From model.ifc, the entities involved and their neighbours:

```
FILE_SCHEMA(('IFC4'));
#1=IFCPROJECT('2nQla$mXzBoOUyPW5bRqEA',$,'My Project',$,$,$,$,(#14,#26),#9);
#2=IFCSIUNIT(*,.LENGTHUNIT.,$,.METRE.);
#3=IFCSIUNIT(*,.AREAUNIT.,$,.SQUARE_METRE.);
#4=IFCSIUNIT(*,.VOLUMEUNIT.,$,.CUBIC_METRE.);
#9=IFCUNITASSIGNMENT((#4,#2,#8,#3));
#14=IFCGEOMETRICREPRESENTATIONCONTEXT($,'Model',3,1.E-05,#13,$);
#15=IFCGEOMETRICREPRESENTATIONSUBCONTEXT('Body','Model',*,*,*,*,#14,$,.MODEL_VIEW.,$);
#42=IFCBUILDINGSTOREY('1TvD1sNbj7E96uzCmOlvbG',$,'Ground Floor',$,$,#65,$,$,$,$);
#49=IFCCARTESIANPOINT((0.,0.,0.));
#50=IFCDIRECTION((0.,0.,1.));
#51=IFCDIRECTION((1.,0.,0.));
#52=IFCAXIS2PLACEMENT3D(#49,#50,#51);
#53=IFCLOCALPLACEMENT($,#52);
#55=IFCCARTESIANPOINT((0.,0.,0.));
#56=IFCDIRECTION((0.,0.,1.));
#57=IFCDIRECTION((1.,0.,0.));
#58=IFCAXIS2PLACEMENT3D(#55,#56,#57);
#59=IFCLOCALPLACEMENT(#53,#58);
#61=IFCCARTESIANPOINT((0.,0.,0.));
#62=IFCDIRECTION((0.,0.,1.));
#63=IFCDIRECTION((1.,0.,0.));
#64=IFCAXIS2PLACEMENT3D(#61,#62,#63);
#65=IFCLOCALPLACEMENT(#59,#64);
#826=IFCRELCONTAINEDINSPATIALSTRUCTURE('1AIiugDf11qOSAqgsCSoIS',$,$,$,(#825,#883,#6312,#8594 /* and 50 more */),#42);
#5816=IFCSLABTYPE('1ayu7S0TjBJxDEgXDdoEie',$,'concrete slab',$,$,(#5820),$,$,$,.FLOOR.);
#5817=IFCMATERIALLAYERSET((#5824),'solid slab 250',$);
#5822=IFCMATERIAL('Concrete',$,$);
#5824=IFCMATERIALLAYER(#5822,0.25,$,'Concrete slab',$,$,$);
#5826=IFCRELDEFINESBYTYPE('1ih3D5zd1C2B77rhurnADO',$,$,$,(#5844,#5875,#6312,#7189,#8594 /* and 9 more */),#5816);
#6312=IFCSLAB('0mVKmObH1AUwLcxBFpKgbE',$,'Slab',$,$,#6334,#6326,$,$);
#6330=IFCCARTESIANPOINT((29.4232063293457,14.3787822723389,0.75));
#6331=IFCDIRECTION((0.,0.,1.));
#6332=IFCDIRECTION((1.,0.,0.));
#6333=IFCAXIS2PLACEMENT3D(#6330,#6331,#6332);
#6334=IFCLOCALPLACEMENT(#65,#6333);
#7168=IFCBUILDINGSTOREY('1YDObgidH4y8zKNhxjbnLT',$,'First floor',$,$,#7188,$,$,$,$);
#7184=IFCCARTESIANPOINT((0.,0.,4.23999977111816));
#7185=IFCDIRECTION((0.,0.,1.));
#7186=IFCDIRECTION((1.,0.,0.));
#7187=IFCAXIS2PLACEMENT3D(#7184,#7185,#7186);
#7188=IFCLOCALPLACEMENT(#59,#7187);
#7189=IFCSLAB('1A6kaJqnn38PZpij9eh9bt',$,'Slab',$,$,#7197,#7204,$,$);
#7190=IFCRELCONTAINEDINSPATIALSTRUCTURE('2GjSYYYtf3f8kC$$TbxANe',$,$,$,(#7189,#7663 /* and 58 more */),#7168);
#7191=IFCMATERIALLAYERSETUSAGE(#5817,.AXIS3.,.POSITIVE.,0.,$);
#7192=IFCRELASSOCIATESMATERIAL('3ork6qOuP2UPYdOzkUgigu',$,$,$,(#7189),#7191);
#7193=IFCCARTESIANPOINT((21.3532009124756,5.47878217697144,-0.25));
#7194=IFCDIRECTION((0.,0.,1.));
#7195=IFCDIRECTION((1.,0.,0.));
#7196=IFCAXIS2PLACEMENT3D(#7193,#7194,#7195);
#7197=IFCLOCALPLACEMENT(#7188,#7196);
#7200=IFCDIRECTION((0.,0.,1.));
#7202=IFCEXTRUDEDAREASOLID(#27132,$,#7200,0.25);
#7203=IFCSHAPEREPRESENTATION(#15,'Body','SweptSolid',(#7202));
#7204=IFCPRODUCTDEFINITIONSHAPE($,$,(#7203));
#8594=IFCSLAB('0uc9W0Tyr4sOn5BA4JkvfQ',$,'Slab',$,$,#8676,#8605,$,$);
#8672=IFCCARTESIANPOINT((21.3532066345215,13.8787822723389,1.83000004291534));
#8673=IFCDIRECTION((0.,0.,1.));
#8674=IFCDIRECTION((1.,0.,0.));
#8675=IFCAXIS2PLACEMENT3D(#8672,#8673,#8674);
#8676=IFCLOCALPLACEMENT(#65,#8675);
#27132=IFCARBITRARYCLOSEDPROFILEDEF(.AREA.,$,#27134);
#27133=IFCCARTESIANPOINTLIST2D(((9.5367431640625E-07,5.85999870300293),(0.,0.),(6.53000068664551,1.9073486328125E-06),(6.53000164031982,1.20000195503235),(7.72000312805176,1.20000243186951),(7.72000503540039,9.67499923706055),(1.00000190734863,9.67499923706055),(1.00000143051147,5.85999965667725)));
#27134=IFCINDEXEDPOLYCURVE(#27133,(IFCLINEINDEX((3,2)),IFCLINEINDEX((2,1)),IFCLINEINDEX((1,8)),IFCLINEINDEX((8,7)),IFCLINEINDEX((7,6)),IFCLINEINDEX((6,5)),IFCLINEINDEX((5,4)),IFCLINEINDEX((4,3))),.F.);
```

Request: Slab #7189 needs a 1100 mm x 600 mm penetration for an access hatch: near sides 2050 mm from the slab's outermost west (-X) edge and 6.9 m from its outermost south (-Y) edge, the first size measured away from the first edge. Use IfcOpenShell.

```python
import numpy as np
import ifcopenshell
import ifcopenshell.api.feature
import ifcopenshell.api.geometry
import ifcopenshell.api.root
import ifcopenshell.geom
import ifcopenshell.util.placement
import ifcopenshell.util.representation
import ifcopenshell.util.shape
import ifcopenshell.util.unit

model = ifcopenshell.open("model.ifc")
unit_scale = ifcopenshell.util.unit.calculate_unit_scale(model)
settings = ifcopenshell.geom.settings()


def volume(element):
    """Net volume in cubic metres, openings subtracted."""
    shape = ifcopenshell.geom.create_shape(settings, element)
    return ifcopenshell.util.shape.get_volume(shape.geometry)


slab = model.by_id(7189)
before = volume(slab)

# Extent in the slab's own axes, in metres. The edges named are its -X and -Y sides.
slab_shape = ifcopenshell.geom.create_shape(settings, slab)
vertices = ifcopenshell.util.shape.get_vertices(slab_shape.geometry)
x_min, y_min, bottom = vertices.min(axis=0)
top = vertices[:, 2].max()

opening = ifcopenshell.api.root.create_entity(model, ifc_class="IfcOpeningElement", name="Access hatch opening", predefined_type="OPENING")
context = ifcopenshell.util.representation.get_context(model, "Model", "Body", "MODEL_VIEW")
width, depth = 1.1, 0.6
outline = [(0.0, 0.0), (width, 0.0), (width, depth), (0.0, depth), (0.0, 0.0)]
# Overshoot both faces by 50 mm so the cut is clean.
shape = ifcopenshell.api.geometry.add_slab_representation(
    model, context=context, depth=top - bottom + 0.1, polyline=outline
)
ifcopenshell.api.geometry.assign_representation(model, product=opening, representation=shape)

matrix = ifcopenshell.util.placement.get_local_placement(slab.ObjectPlacement)
matrix[:, 3] = matrix @ np.append(np.array([x_min + 2.05, y_min + 6.9, bottom - 0.05]) / unit_scale, 1.0)
ifcopenshell.api.geometry.edit_object_placement(model, product=opening, matrix=matrix, is_si=False)
ifcopenshell.api.feature.add_feature(model, feature=opening, element=slab)

after = volume(slab)

print(f"slab volume {before:.3f} -> {after:.3f} m3")

model.write("model-out.ifc")
```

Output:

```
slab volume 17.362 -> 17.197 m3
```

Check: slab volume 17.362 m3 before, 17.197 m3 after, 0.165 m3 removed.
